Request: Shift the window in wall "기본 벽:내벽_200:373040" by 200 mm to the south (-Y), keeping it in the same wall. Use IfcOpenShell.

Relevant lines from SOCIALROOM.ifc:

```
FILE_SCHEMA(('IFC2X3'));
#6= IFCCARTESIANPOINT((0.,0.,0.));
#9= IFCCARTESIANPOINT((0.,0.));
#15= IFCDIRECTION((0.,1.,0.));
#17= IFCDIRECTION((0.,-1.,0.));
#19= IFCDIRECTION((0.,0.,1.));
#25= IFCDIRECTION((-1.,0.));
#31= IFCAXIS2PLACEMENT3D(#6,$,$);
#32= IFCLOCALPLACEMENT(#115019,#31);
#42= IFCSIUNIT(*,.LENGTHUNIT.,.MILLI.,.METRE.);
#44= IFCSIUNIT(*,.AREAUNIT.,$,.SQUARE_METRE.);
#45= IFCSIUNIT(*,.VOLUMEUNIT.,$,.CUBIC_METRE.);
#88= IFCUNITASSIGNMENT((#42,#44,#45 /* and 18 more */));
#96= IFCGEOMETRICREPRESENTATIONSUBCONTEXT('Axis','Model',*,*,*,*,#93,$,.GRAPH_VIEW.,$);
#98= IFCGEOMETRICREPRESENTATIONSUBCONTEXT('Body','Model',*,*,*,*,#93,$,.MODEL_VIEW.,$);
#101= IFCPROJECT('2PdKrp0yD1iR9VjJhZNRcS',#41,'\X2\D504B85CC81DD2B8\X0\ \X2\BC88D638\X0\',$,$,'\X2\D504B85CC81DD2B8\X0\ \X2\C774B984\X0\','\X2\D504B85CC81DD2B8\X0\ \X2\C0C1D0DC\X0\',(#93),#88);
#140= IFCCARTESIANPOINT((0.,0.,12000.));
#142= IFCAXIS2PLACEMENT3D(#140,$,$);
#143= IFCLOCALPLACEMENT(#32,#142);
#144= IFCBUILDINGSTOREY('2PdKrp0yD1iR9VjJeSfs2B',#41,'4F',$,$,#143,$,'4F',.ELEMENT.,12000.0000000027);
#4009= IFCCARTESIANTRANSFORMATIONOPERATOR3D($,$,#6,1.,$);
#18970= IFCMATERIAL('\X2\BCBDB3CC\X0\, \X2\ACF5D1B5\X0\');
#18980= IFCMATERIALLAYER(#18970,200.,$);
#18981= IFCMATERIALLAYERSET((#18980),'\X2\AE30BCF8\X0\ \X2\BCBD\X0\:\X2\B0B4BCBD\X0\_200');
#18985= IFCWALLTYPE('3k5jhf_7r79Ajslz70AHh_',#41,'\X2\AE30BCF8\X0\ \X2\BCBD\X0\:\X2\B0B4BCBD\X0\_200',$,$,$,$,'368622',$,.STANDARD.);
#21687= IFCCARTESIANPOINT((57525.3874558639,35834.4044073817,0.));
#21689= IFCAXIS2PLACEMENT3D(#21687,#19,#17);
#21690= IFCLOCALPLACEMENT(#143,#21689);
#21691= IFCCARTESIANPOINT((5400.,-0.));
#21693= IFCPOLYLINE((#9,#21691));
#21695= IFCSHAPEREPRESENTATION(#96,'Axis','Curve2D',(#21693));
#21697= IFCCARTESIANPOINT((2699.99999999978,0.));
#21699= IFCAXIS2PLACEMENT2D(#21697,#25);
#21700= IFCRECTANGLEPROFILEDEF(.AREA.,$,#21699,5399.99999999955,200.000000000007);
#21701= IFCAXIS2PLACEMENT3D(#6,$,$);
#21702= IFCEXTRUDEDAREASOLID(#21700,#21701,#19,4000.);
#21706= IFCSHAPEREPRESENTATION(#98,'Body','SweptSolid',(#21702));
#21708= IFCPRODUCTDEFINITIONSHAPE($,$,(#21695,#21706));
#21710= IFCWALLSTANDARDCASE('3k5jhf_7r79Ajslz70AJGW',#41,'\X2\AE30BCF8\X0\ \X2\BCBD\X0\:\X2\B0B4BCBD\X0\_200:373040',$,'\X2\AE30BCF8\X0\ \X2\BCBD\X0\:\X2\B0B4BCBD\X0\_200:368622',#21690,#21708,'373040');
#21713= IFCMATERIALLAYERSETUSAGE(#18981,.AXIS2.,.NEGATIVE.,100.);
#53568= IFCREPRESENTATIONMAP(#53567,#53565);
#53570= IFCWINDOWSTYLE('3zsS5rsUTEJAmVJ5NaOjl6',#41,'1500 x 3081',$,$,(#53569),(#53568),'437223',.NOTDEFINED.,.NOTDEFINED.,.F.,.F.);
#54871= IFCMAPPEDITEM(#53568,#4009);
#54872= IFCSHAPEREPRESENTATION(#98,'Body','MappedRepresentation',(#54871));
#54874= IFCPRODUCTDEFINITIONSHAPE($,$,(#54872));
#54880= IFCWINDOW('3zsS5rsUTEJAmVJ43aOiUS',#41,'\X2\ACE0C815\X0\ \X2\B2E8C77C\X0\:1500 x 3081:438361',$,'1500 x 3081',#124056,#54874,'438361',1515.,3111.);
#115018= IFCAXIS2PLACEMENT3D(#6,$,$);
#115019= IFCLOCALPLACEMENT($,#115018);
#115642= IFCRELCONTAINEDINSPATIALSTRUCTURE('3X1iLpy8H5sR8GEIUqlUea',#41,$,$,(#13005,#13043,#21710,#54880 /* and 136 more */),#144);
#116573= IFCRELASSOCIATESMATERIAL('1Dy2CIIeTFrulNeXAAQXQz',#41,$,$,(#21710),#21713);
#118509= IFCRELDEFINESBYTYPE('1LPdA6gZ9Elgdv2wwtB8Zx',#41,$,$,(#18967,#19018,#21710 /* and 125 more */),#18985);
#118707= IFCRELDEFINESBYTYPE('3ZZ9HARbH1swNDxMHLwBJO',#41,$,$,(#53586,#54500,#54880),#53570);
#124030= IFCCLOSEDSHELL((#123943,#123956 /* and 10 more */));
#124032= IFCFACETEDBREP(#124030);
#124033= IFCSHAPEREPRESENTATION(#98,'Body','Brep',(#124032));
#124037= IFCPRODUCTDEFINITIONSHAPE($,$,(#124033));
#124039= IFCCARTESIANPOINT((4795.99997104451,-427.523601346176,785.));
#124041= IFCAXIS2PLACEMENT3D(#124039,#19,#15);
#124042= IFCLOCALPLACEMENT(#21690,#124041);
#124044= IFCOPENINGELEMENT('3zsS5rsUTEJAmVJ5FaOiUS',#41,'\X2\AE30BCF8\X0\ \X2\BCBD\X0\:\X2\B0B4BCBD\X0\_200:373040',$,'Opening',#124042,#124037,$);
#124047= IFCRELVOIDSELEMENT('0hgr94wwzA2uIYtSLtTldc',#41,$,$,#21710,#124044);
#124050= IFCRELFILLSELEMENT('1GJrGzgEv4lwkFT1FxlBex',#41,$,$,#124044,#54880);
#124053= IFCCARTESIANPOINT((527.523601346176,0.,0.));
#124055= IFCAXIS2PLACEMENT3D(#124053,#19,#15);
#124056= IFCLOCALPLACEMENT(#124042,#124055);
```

```python
import ifcopenshell
import ifcopenshell.api.geometry
import ifcopenshell.util.placement

model = ifcopenshell.open("SOCIALROOM.ifc")

window = model.by_id(54880)
opening = window.FillsVoids[0].RelatingOpeningElement
wall = opening.VoidsElements[0].RelatingBuildingElement

wall_matrix = ifcopenshell.util.placement.get_local_placement(wall.ObjectPlacement)
shift = wall_matrix[:3, 0] * 200.0
before = ifcopenshell.util.placement.get_local_placement(window.ObjectPlacement)[:3, 3].copy()

# The window is placed relative to its opening, so it follows when the opening moves.
matrix = ifcopenshell.util.placement.get_local_placement(opening.ObjectPlacement)
matrix[:3, 3] += shift
ifcopenshell.api.geometry.edit_object_placement(
    model, product=opening, matrix=matrix, is_si=False, should_transform_children=True
)

after = ifcopenshell.util.placement.get_local_placement(window.ObjectPlacement)[:3, 3]
print("window moved by", (after - before).round(3) + 0.0)

model.write("SOCIALROOM-out.ifc")
```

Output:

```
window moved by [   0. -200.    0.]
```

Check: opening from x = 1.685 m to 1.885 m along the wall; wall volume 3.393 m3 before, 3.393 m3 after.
